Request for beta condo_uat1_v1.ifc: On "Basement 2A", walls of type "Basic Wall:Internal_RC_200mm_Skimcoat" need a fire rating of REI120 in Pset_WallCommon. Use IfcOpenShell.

First a look at what the model holds.

```python
import ifcopenshell
import ifcopenshell.util.element

model = ifcopenshell.open("beta condo_uat1_v1.ifc")
print(model.schema)
storey = next(s for s in model.by_type("IfcBuildingStorey") if s.Name == "Basement 2A")
walls = [e for e in ifcopenshell.util.element.get_decomposition(storey) if e.is_a("IfcWall")]
seen = {}
for e in walls:
    element_type = ifcopenshell.util.element.get_type(e)
    key = (element_type.Name if element_type != e and element_type else None, ifcopenshell.util.element.get_pset(e, "Pset_WallCommon", "FireRating"))
    seen[key] = seen.get(key, 0) + 1
for (name, value), count in sorted(seen.items(), key=str):
    print(count, "x", name, "|", value)
```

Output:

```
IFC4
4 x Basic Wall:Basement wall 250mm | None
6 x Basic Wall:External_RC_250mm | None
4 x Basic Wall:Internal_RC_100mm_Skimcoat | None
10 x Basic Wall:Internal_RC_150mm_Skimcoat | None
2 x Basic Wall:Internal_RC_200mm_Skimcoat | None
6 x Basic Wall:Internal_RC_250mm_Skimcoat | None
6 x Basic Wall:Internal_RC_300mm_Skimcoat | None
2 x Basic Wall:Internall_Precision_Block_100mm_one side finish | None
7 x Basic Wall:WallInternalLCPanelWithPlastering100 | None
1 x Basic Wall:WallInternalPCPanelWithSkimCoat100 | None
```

```python
import ifcopenshell
import ifcopenshell.api.pset
import ifcopenshell.util.element

model = ifcopenshell.open("beta condo_uat1_v1.ifc")

storey = next(s for s in model.by_type("IfcBuildingStorey") if s.Name == "Basement 2A")
walls = [e for e in ifcopenshell.util.element.get_decomposition(storey) if e.is_a("IfcWall")]

count = 0
for e in walls:
    element_type = ifcopenshell.util.element.get_type(e)
    if element_type in (None, e) or element_type.Name != "Basic Wall:Internal_RC_200mm_Skimcoat":
        continue
    # add_pset returns the element's existing set when there is one.
    pset = ifcopenshell.api.pset.add_pset(model, product=e, name="Pset_WallCommon")
    ifcopenshell.api.pset.edit_pset(model, pset=pset, properties={"FireRating": "REI120"})
    count += 1

print(count, "walls updated")

model.write("beta condo_uat1_v1-out.ifc")
```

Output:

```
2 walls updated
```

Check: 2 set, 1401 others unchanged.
